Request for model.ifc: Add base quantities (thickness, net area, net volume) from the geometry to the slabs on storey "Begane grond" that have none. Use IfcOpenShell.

First a look at what the model holds.

```python
import ifcopenshell
import ifcopenshell.util.element
import ifcopenshell.util.unit

model = ifcopenshell.open("model.ifc")
print(model.schema)
for unit_type in ("LENGTHUNIT", "AREAUNIT", "VOLUMEUNIT"):
    print(unit_type, ifcopenshell.util.unit.calculate_unit_scale(model, unit_type))
storey = next(s for s in model.by_type("IfcBuildingStorey") if s.Name == "Begane grond")
slabs = [e for e in ifcopenshell.util.element.get_decomposition(storey) if e.is_a("IfcSlab")]
for e in sorted(slabs, key=lambda e: e.id()):
    print(e.id(), e.is_a(), e.Name, list(ifcopenshell.util.element.get_psets(e, qtos_only=True)), sep=" | ")
```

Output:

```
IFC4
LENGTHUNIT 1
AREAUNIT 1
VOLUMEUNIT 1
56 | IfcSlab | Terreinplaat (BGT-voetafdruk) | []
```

```python
import ifcopenshell
import ifcopenshell.api.pset
import ifcopenshell.geom
import ifcopenshell.util.element
import ifcopenshell.util.shape
import ifcopenshell.util.unit

model = ifcopenshell.open("model.ifc")
unit_scale = ifcopenshell.util.unit.calculate_unit_scale(model)
area_scale = ifcopenshell.util.unit.calculate_unit_scale(model, "AREAUNIT")
volume_scale = ifcopenshell.util.unit.calculate_unit_scale(model, "VOLUMEUNIT")
settings = ifcopenshell.geom.settings()

storey = next(s for s in model.by_type("IfcBuildingStorey") if s.Name == "Begane grond")
slabs = [e for e in ifcopenshell.util.element.get_decomposition(storey) if e.is_a("IfcSlab")]

for e in sorted(slabs, key=lambda e: e.id()):
    if ifcopenshell.util.element.get_psets(e, qtos_only=True, should_inherit=False):
        continue
    # Geometry comes back in metres, in the element's own axes.
    shape = ifcopenshell.geom.create_shape(settings, e)
    values = {
        "Width": ifcopenshell.util.shape.get_z(shape.geometry) / unit_scale,
        "NetArea": ifcopenshell.util.shape.get_footprint_area(shape.geometry) / area_scale,
        "NetVolume": ifcopenshell.util.shape.get_volume(shape.geometry) / volume_scale,
    }
    qto = ifcopenshell.api.pset.add_qto(model, product=e, name="Qto_SlabBaseQuantities")
    ifcopenshell.api.pset.edit_qto(model, qto=qto, properties=values)
    print(e.id(), {k: round(v, 3) for k, v in values.items()})

model.write("model_v2.ifc")
```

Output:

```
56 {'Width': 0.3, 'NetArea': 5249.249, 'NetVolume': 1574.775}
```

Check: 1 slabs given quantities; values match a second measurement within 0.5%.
